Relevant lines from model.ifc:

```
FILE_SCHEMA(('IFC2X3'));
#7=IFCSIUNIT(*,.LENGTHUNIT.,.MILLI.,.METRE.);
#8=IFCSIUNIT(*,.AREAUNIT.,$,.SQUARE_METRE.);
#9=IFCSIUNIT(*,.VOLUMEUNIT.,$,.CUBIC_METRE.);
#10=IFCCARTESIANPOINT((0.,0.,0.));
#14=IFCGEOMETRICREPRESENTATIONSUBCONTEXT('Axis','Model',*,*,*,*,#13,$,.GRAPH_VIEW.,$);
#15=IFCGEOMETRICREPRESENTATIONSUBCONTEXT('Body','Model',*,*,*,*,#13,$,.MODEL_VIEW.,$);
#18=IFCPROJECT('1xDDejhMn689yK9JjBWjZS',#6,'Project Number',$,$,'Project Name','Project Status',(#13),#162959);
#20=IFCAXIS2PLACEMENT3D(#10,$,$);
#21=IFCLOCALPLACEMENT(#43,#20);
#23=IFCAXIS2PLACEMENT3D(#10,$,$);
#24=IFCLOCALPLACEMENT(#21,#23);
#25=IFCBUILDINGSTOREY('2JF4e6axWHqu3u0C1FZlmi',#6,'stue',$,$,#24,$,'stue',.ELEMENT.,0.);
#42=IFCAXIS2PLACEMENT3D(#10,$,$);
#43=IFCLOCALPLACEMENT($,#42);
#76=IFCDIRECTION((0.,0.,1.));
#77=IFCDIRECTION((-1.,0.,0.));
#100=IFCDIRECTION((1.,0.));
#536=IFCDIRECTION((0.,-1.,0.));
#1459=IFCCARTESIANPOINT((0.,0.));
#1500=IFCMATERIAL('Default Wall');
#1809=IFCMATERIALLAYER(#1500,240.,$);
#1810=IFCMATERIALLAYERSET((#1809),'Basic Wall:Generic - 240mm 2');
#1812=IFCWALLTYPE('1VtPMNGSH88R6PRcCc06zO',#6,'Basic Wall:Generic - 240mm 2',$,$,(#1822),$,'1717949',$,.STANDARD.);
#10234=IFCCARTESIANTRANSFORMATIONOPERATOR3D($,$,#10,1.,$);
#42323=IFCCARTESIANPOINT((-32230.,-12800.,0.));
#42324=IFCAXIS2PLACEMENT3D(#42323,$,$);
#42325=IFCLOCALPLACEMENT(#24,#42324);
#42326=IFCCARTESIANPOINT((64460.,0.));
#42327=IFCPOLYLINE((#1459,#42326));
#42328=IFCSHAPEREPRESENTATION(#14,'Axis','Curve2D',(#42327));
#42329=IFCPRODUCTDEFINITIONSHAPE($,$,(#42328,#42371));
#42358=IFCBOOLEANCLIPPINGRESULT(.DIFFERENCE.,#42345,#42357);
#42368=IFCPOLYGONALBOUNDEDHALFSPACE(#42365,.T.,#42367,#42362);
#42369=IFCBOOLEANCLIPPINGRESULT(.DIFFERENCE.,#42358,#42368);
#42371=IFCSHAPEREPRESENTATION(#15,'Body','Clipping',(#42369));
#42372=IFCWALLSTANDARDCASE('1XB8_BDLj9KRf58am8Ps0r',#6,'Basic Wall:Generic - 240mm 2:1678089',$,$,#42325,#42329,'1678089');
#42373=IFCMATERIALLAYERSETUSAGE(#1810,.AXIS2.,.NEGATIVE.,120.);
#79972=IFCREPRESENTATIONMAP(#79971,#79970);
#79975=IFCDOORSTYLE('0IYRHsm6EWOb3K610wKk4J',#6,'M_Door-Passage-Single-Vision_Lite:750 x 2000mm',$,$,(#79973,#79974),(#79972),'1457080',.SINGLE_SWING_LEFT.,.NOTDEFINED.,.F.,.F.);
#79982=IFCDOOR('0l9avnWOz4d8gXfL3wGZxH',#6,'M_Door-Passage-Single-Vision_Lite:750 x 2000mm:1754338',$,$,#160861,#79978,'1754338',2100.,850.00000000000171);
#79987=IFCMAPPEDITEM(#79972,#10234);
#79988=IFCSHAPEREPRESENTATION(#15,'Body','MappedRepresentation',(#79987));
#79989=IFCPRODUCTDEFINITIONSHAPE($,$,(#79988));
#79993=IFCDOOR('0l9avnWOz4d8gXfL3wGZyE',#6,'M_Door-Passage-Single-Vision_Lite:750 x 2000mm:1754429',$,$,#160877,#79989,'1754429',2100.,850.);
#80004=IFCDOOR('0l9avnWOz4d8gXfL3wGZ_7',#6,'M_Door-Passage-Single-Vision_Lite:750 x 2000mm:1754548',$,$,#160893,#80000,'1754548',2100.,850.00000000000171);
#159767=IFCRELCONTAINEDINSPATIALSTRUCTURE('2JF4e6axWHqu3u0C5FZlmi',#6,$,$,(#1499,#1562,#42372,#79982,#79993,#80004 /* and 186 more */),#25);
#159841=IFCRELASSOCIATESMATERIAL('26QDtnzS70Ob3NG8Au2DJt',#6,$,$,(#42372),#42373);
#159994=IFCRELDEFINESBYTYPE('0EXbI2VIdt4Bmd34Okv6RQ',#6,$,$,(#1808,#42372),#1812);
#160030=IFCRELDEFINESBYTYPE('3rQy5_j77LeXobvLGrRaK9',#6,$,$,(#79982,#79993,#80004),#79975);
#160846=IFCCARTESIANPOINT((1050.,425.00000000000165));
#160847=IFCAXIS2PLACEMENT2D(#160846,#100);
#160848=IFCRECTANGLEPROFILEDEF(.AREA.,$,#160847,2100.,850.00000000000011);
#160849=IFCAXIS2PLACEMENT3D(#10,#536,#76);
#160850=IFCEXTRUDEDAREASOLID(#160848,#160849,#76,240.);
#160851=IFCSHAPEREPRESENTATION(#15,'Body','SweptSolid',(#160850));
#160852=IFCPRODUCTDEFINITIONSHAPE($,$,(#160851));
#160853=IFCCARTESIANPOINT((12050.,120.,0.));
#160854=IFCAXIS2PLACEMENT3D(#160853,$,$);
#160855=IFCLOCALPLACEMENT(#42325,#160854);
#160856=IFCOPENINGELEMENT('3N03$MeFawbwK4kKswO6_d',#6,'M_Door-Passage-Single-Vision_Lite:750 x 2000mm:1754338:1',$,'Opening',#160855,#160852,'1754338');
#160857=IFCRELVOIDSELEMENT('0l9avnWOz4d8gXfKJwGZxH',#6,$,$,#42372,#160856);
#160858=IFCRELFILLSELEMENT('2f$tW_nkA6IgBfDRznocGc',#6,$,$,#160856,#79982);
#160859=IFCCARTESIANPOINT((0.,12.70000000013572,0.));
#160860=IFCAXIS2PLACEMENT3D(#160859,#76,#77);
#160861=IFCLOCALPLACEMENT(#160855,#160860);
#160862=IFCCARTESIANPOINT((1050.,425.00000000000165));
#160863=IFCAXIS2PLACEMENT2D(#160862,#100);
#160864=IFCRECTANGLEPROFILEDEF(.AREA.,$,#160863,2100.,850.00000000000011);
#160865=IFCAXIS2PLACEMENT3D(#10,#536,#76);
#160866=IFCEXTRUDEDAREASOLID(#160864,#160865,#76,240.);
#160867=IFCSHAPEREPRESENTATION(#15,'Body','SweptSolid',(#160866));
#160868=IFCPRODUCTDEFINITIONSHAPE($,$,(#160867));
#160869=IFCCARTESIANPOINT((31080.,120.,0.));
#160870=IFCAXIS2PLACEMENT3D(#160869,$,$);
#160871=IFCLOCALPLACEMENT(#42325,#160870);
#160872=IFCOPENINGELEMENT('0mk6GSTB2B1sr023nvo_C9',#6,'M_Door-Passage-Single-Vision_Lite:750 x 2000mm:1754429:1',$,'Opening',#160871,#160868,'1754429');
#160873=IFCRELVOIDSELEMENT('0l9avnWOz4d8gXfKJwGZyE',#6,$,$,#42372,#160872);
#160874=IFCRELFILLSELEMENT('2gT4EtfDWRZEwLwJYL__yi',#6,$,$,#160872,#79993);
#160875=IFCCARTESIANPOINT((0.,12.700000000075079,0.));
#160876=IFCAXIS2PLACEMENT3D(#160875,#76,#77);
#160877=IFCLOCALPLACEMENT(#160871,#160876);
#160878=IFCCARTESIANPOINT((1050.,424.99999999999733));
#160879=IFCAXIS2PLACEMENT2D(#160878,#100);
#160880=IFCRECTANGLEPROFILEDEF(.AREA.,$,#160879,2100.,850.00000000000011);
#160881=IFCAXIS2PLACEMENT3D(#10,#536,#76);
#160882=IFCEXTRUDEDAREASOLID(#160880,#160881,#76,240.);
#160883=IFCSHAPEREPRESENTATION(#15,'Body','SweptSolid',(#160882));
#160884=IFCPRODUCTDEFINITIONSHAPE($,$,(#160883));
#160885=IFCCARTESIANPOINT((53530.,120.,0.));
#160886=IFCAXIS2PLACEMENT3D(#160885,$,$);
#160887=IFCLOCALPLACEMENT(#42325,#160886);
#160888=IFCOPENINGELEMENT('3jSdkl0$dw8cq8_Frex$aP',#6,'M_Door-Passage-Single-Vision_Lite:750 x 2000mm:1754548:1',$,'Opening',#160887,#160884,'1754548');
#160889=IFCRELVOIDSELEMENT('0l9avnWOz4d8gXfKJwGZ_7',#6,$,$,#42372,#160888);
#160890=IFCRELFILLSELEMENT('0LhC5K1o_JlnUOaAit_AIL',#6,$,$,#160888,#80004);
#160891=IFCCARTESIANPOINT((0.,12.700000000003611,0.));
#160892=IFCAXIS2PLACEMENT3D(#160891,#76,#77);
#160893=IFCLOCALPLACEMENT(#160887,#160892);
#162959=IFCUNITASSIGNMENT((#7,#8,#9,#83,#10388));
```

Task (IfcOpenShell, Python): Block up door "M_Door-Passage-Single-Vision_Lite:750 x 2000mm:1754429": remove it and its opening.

```python
import ifcopenshell
import ifcopenshell.api.feature
import ifcopenshell.api.root
import ifcopenshell.geom
import ifcopenshell.util.shape

model = ifcopenshell.open("model.ifc")
settings = ifcopenshell.geom.settings()


def volume(element):
    """Net volume in cubic metres, openings subtracted."""
    shape = ifcopenshell.geom.create_shape(settings, element)
    return ifcopenshell.util.shape.get_volume(shape.geometry)


door = model.by_guid("0l9avnWOz4d8gXfL3wGZyE")
opening = door.FillsVoids[0].RelatingOpeningElement
wall = opening.VoidsElements[0].RelatingBuildingElement
before = volume(wall)

ifcopenshell.api.root.remove_product(model, product=door)
ifcopenshell.api.feature.remove_feature(model, feature=opening)

after = volume(wall)

print(f"wall volume {before:.3f} -> {after:.3f} m3")

model.write("model_edited.ifc")
```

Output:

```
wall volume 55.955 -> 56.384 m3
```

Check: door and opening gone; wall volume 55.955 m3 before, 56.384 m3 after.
